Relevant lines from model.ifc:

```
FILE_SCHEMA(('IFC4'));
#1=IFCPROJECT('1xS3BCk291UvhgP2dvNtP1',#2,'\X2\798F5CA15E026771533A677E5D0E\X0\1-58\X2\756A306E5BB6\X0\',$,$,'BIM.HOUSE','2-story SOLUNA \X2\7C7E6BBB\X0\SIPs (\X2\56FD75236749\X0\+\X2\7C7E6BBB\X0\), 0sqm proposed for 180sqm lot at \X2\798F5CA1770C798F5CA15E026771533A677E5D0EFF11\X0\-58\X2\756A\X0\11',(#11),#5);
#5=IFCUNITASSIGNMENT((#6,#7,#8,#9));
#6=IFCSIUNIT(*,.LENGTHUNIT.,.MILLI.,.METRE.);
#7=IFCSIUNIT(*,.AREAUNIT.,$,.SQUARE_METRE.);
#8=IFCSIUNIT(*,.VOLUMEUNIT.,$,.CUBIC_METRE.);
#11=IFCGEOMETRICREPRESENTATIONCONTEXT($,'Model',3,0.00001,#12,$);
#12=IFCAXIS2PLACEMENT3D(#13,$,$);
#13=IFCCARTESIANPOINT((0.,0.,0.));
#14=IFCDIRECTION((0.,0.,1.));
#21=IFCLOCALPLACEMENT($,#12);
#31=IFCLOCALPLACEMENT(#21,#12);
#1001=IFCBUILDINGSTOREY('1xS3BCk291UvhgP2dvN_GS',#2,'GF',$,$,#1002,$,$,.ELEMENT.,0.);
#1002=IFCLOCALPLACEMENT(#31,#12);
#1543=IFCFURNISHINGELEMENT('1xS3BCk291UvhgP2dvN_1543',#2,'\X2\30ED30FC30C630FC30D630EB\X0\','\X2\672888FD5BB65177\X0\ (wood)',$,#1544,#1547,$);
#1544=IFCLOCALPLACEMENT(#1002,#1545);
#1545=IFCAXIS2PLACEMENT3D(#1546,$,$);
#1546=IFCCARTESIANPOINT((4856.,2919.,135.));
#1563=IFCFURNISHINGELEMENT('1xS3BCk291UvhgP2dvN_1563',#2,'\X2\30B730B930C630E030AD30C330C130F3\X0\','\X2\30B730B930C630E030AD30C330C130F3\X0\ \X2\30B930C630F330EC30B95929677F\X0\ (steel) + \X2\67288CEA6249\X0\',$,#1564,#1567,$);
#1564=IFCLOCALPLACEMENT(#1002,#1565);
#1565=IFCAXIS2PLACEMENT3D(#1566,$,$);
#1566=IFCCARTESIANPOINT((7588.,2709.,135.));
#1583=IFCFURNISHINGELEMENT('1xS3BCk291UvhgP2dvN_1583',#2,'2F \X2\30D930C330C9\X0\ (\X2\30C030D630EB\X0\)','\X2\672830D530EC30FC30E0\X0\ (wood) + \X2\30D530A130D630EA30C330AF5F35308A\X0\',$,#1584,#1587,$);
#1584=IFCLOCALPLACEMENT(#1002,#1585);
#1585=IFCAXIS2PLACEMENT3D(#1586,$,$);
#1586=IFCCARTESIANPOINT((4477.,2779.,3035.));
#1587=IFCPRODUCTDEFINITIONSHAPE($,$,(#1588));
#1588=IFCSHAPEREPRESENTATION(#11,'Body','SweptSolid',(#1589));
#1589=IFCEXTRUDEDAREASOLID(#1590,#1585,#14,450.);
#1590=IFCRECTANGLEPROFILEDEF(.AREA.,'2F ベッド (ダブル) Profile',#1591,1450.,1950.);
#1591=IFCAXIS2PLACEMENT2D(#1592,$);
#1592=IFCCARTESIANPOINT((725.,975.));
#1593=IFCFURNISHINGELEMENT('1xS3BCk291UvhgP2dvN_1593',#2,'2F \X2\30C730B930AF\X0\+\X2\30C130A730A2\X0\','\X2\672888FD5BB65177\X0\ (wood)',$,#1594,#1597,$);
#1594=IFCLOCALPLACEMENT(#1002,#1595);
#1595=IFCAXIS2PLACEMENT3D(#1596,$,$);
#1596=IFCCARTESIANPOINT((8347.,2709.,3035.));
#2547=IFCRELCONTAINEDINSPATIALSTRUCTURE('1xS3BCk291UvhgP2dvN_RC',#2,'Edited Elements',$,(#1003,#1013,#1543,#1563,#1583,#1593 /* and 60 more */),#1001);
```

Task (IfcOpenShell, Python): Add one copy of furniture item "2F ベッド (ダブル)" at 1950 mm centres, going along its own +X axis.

```python
import ifcopenshell
import ifcopenshell.api.geometry
import ifcopenshell.api.root
import ifcopenshell.util.element
import ifcopenshell.util.placement
import ifcopenshell.util.unit

model = ifcopenshell.open("model.ifc")
unit_scale = ifcopenshell.util.unit.calculate_unit_scale(model)


def reuse_history(source, copy):
    """copy_class also copies each property set's owner history, people and application; keep the originals."""
    for rel in copy.IsDefinedBy:
        if rel.is_a("IfcRelDefinesByProperties") and (history := rel.RelatingPropertyDefinition.OwnerHistory):
            rel.RelatingPropertyDefinition.OwnerHistory = source.OwnerHistory
            ifcopenshell.util.element.remove_deep2(model, history)


source = model.by_id(1583)
base = ifcopenshell.util.placement.get_local_placement(source.ObjectPlacement)
step = base[:3, 0] * 1.95 / unit_scale

for i in range(1, 2):
    copy = ifcopenshell.api.root.copy_class(model, product=source)
    copy.Representation = ifcopenshell.util.element.copy_deep(
        model, source.Representation, exclude=["IfcGeometricRepresentationContext", "IfcRepresentationMap"]
    )
    reuse_history(source, copy)
    matrix = base.copy()
    matrix[:3, 3] += i * step
    print("added at", matrix[:3, 3].round(3) + 0.0)
    ifcopenshell.api.geometry.edit_object_placement(model, product=copy, matrix=matrix, is_si=False)

model.write("model_v2.ifc")
```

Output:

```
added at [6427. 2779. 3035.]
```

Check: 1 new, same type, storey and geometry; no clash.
